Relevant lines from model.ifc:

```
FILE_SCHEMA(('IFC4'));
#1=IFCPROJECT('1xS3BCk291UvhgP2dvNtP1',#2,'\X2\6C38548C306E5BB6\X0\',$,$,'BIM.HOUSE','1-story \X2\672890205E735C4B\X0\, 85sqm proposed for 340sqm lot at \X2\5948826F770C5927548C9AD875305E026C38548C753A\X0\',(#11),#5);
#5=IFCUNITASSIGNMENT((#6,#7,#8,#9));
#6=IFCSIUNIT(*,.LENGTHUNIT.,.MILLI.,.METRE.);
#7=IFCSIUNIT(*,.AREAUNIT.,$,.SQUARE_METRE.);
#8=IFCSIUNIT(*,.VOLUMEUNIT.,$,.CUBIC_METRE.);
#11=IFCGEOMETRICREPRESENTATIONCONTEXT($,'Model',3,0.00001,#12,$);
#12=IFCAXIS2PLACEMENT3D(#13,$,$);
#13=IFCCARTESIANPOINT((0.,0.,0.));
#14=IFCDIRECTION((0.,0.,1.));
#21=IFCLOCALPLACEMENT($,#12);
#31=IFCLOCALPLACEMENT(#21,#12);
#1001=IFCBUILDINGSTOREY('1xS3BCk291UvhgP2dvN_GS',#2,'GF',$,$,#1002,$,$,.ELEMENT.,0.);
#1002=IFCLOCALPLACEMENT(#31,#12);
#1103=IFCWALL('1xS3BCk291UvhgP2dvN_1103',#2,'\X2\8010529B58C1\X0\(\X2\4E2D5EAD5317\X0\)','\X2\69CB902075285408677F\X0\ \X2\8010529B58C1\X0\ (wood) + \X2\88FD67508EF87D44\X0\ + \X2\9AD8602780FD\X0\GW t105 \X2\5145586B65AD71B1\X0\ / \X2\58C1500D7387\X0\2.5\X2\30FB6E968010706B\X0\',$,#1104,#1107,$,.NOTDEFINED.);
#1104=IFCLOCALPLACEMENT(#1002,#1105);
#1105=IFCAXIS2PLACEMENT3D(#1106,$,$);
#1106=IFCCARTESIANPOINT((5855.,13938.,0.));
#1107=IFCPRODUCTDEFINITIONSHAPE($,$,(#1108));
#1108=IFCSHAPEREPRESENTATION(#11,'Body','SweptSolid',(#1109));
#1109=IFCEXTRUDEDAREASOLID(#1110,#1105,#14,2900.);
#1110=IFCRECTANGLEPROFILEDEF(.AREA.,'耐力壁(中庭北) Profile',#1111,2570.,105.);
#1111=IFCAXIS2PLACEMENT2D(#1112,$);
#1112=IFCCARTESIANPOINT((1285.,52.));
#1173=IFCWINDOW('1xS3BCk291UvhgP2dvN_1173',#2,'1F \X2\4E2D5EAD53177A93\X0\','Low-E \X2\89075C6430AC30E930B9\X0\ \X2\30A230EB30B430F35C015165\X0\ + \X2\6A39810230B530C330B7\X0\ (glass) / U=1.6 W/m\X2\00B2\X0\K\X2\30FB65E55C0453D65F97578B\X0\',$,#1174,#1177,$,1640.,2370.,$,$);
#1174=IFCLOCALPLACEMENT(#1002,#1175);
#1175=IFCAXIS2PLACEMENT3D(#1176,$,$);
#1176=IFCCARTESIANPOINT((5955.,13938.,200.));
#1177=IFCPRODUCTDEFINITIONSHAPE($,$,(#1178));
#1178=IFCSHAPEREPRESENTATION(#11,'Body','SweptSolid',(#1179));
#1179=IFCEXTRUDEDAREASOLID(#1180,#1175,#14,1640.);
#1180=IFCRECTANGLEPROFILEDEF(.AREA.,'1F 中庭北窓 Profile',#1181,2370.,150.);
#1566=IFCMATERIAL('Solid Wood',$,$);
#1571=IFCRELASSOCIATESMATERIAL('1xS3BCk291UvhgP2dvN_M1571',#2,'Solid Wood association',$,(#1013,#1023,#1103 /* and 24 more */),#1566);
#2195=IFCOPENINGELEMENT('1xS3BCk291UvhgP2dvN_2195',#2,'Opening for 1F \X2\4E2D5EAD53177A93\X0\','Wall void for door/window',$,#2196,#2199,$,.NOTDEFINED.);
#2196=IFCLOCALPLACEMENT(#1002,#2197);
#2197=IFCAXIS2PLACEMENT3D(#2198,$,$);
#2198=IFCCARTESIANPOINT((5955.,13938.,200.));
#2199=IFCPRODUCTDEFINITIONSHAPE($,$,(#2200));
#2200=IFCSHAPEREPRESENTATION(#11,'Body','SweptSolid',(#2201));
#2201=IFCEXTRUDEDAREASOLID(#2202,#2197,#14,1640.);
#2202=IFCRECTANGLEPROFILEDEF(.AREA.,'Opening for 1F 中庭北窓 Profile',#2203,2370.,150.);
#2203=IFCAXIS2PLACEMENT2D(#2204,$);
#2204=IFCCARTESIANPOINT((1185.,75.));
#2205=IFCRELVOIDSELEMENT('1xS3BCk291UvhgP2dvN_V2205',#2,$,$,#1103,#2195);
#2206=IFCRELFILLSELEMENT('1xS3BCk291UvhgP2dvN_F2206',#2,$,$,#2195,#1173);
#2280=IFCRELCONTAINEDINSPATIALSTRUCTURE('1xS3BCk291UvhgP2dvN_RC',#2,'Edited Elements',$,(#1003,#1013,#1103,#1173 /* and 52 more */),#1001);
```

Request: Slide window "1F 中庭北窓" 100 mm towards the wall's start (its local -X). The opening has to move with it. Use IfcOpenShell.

```python
import ifcopenshell
import ifcopenshell.api.geometry
import ifcopenshell.util.placement

model = ifcopenshell.open("model.ifc")

window = model.by_id(1173)
opening = window.FillsVoids[0].RelatingOpeningElement
wall = opening.VoidsElements[0].RelatingBuildingElement

wall_matrix = ifcopenshell.util.placement.get_local_placement(wall.ObjectPlacement)
shift = wall_matrix[:3, 0] * -100.0
before = ifcopenshell.util.placement.get_local_placement(window.ObjectPlacement)[:3, 3].copy()

# The window is not placed relative to its opening, so move both.
for product in (opening, window):
    matrix = ifcopenshell.util.placement.get_local_placement(product.ObjectPlacement)
    matrix[:3, 3] += shift
    ifcopenshell.api.geometry.edit_object_placement(model, product=product, matrix=matrix, is_si=False)

after = ifcopenshell.util.placement.get_local_placement(window.ObjectPlacement)[:3, 3]
print("window moved by", (after - before).round(3) + 0.0)

model.write("model-out.ifc")
```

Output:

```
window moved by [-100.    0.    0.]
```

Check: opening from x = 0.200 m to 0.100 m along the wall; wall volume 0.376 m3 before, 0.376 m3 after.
